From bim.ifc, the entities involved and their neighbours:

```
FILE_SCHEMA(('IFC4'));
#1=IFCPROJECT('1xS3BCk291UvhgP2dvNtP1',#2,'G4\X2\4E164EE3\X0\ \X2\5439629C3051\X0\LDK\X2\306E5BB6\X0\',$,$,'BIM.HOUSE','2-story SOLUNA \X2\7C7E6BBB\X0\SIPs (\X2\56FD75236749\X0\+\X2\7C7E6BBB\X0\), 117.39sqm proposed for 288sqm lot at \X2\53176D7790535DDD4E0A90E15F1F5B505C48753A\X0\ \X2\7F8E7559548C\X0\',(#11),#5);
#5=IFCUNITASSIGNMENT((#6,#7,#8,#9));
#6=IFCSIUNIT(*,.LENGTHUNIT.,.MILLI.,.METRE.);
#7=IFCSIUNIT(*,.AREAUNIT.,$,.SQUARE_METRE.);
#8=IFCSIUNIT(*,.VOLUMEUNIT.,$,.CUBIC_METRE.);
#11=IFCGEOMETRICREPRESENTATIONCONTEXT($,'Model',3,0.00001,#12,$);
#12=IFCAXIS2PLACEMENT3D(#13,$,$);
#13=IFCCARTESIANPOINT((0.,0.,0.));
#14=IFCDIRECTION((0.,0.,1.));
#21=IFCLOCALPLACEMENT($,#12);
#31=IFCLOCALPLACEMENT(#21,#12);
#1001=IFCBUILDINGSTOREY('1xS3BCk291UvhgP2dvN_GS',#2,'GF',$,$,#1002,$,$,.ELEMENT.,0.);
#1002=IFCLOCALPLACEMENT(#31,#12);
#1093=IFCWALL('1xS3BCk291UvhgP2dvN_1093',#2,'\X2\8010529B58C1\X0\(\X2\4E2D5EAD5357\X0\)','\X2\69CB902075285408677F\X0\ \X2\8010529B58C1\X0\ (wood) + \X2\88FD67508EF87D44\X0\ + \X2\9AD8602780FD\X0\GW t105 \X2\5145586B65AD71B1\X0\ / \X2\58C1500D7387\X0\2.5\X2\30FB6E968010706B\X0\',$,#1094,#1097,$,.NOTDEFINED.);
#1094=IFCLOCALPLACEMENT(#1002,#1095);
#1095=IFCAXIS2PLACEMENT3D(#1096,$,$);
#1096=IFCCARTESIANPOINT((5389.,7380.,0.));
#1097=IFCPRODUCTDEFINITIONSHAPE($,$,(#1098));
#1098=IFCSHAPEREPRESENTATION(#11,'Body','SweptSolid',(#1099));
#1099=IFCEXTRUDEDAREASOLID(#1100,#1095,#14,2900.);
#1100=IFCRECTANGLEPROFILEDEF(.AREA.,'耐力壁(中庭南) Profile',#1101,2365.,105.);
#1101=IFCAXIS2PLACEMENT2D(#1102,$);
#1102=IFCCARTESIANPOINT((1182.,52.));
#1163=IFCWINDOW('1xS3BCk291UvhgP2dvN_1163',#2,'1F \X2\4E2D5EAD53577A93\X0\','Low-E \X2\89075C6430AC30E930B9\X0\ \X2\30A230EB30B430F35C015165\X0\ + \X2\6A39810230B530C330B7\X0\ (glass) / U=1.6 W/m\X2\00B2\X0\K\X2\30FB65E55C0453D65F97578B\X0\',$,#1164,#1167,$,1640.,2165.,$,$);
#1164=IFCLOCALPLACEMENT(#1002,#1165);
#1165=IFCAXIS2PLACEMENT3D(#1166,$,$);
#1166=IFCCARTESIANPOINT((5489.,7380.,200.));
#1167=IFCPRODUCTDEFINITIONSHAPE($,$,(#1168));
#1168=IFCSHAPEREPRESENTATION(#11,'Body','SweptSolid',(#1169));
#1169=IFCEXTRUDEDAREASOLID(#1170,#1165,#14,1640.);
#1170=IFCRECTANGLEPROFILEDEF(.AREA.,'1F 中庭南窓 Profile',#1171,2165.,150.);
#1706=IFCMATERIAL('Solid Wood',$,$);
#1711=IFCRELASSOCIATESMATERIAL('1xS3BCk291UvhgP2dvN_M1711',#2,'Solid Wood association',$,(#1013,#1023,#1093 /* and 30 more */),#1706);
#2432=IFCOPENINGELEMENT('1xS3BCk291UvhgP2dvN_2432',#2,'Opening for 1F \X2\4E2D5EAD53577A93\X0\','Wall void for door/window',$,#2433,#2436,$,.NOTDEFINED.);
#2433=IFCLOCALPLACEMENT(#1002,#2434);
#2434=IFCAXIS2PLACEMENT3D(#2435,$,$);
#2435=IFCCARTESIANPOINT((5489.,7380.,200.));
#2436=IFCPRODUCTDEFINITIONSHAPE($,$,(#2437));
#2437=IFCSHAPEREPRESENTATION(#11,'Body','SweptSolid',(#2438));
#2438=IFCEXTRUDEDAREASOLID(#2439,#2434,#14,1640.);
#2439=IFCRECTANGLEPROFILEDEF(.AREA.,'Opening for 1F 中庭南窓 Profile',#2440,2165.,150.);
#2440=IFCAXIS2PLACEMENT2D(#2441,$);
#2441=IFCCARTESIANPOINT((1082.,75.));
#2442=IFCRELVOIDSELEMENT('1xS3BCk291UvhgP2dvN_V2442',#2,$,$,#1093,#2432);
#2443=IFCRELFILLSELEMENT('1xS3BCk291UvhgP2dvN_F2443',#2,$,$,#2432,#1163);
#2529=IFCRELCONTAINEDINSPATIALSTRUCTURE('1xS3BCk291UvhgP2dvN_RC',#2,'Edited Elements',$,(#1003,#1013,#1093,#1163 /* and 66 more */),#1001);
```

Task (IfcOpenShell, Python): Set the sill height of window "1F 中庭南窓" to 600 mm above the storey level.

```python
import numpy as np
import ifcopenshell
import ifcopenshell.api.geometry
import ifcopenshell.geom
import ifcopenshell.util.element
import ifcopenshell.util.placement
import ifcopenshell.util.shape
import ifcopenshell.util.unit

model = ifcopenshell.open("bim.ifc")
unit_scale = ifcopenshell.util.unit.calculate_unit_scale(model)

window = model.by_guid("1xS3BCk291UvhgP2dvN_1163")
opening = window.FillsVoids[0].RelatingOpeningElement
storey = ifcopenshell.util.element.get_container(window, ifc_class="IfcBuildingStorey")
level = ifcopenshell.util.placement.get_local_placement(storey.ObjectPlacement)[2, 3]

# The opening's origin need not be at the sill, so measure its lowest point.
shape = ifcopenshell.geom.create_shape(ifcopenshell.geom.settings(), opening)
bottom = ifcopenshell.util.shape.get_shape_bottom_elevation(shape, shape.geometry) / unit_scale
dz = level + 600.0 - bottom

shift = np.array([0.0, 0.0, dz])
# The window is not placed relative to its opening, so move both.
for product in (opening, window):
    matrix = ifcopenshell.util.placement.get_local_placement(product.ObjectPlacement)
    matrix[:3, 3] += shift
    ifcopenshell.api.geometry.edit_object_placement(model, product=product, matrix=matrix, is_si=False)

print(f"moved by {dz * unit_scale:+.3f} m")

model.write("bim_rev.ifc")
```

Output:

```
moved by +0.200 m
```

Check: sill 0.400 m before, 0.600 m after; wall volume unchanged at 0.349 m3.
